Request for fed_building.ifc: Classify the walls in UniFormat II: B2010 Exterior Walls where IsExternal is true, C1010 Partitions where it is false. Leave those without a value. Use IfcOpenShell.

First a look at what the model holds.

```python
import ifcopenshell
import ifcopenshell.util.element

model = ifcopenshell.open("fed_building.ifc")
print(model.schema)
print("classifications:", [c.Name for c in model.by_type("IfcClassification")])
values = [ifcopenshell.util.element.get_pset(e, "Pset_WallCommon", "IsExternal") for e in model.by_type("IfcWall")]
for value in (True, False, None):
    print("IsExternal", value, values.count(value))
```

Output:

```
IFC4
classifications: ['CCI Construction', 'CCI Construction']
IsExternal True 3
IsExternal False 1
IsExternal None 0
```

```python
import ifcopenshell
import ifcopenshell.api.classification
import ifcopenshell.util.element

model = ifcopenshell.open("fed_building.ifc")

system = ifcopenshell.api.classification.add_classification(model, classification="UniFormat II")

walls = model.by_type("IfcWall")
external = {e: ifcopenshell.util.element.get_pset(e, "Pset_WallCommon", "IsExternal") for e in walls}
for flag, code, name in ((True, "B2010", "Exterior Walls"), (False, "C1010", "Partitions")):
    products = [e for e in walls if external[e] is flag]
    ifcopenshell.api.classification.add_reference(
        model, products=products, classification=system, identification=code, name=name
    )
    print(code, len(products))

model.write("fed_building_updated.ifc")
```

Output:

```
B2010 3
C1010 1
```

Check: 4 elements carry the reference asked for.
